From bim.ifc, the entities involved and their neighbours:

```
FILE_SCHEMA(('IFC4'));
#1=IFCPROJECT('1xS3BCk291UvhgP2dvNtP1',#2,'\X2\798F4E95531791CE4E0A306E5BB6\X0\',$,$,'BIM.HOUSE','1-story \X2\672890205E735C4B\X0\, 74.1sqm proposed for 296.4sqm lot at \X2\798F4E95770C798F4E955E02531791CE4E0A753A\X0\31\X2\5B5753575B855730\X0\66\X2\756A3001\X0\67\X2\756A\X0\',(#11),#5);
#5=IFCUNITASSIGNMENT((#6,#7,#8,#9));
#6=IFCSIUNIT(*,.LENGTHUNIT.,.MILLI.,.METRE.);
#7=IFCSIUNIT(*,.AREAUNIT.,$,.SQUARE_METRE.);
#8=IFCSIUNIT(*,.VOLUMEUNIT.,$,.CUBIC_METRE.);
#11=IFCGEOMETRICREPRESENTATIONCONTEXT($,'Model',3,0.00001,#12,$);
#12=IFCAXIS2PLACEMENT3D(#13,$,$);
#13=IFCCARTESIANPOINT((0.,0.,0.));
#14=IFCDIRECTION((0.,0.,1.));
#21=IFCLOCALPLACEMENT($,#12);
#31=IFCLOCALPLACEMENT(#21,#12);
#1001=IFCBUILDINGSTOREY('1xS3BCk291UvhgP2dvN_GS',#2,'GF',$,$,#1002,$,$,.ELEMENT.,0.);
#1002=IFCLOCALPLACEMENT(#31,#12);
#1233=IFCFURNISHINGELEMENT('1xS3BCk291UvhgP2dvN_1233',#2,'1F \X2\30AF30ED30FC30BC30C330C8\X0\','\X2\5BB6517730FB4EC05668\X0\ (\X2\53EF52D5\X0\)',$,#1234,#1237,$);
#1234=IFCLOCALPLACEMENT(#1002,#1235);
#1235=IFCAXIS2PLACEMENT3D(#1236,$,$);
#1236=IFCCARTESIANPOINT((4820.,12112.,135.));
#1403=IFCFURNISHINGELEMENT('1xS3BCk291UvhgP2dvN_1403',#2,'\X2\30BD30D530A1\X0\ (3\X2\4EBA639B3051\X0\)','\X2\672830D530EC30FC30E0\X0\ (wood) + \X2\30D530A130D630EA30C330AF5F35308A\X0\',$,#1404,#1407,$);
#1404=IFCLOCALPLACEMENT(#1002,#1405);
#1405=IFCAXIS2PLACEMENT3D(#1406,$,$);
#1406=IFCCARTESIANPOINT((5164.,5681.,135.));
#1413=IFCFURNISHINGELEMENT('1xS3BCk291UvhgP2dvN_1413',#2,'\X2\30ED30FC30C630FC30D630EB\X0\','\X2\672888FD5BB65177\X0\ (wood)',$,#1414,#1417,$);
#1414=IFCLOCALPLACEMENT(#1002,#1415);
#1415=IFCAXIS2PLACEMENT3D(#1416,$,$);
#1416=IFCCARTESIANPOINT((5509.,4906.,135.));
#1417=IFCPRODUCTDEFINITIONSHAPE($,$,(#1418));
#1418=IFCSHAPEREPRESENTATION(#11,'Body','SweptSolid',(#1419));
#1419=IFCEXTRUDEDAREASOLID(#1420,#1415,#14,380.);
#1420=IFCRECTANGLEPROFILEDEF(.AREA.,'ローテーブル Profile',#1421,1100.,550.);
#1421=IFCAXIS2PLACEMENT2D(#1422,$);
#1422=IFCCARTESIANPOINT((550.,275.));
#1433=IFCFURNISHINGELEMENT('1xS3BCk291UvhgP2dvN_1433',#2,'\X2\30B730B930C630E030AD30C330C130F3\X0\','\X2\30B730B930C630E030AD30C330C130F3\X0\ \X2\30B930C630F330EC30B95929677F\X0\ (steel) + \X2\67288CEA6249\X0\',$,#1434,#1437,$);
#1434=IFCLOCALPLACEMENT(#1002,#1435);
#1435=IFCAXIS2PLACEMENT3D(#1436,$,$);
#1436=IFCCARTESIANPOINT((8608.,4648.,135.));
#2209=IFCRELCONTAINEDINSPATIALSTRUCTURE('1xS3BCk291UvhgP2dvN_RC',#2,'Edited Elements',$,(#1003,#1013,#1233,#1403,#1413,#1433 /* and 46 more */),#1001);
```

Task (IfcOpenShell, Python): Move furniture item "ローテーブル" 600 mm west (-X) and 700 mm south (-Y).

```python
import ifcopenshell
import ifcopenshell.api.geometry
import ifcopenshell.util.placement
import ifcopenshell.util.unit

model = ifcopenshell.open("bim.ifc")
unit_scale = ifcopenshell.util.unit.calculate_unit_scale(model)

item = model.by_guid("1xS3BCk291UvhgP2dvN_1413")
matrix = ifcopenshell.util.placement.get_local_placement(item.ObjectPlacement)
matrix[0, 3] -= 0.6 / unit_scale
matrix[1, 3] -= 0.7 / unit_scale
ifcopenshell.api.geometry.edit_object_placement(model, product=item, matrix=matrix, is_si=False)

print(ifcopenshell.util.placement.get_local_placement(item.ObjectPlacement).round(3) + 0.0)

model.write("bim_v2.ifc")
```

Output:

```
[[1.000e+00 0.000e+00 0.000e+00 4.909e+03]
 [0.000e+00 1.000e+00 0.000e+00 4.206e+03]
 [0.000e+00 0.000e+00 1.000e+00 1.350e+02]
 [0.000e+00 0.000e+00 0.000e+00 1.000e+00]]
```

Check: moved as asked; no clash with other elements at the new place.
